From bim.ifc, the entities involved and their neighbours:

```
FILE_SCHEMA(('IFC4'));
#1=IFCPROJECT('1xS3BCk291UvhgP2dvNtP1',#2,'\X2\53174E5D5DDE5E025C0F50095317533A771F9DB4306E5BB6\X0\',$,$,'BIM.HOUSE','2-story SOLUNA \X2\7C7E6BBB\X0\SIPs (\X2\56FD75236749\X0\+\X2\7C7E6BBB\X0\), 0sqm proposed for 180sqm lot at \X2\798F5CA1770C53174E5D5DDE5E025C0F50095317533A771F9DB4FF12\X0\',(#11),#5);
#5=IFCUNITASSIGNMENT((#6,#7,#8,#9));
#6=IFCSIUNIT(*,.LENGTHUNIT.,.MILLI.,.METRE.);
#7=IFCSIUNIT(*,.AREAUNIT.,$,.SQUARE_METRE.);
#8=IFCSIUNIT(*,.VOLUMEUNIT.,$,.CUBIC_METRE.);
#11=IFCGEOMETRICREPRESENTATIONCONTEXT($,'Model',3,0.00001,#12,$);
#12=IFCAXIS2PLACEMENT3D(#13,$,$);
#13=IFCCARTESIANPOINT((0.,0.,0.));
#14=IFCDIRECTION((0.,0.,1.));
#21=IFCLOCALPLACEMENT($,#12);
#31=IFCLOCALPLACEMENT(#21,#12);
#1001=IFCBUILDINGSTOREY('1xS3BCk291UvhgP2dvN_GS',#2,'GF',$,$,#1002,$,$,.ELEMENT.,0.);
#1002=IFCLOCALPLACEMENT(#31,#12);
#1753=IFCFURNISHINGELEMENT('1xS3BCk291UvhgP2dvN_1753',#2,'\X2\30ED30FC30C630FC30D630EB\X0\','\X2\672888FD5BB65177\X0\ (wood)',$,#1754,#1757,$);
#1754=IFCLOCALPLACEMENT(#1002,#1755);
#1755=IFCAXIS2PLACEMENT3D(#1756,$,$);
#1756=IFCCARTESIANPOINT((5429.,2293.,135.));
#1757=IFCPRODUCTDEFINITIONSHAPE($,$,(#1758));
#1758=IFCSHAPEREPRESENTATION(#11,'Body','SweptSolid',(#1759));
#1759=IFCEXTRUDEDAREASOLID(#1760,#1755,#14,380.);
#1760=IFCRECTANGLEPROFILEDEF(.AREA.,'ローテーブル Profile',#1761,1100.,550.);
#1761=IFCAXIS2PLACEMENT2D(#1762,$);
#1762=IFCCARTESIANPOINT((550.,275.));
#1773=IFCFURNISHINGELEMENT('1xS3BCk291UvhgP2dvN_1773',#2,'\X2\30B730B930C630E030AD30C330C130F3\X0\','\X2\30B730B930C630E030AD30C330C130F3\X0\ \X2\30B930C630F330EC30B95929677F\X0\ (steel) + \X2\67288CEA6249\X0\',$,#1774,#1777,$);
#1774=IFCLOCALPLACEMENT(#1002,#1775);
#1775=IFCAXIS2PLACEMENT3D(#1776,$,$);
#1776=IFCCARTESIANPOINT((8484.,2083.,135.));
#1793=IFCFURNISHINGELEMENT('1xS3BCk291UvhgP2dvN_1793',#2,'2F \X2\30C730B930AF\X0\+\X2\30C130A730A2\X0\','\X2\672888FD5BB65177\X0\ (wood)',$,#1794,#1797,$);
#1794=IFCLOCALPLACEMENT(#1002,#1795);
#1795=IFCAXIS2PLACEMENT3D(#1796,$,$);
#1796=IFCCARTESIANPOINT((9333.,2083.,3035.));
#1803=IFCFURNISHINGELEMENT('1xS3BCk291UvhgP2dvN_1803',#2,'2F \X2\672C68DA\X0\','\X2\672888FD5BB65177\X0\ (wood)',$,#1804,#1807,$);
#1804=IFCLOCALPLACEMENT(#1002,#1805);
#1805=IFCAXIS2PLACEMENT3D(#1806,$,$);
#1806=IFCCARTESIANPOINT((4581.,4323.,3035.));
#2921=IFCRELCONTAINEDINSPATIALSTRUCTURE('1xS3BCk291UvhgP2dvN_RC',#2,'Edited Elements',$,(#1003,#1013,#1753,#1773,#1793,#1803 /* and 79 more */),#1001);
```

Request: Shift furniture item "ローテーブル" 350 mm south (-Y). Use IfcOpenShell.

```python
import ifcopenshell
import ifcopenshell.api.geometry
import ifcopenshell.util.placement
import ifcopenshell.util.unit

model = ifcopenshell.open("bim.ifc")
unit_scale = ifcopenshell.util.unit.calculate_unit_scale(model)

item = model.by_guid("1xS3BCk291UvhgP2dvN_1753")
matrix = ifcopenshell.util.placement.get_local_placement(item.ObjectPlacement)
matrix[1, 3] -= 0.35 / unit_scale
ifcopenshell.api.geometry.edit_object_placement(model, product=item, matrix=matrix, is_si=False)

print(ifcopenshell.util.placement.get_local_placement(item.ObjectPlacement).round(3) + 0.0)

model.write("bim_rev.ifc")
```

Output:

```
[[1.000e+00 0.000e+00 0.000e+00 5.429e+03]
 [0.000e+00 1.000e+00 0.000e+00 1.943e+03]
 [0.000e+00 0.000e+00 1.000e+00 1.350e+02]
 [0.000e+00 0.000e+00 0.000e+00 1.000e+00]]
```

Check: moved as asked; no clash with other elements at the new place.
